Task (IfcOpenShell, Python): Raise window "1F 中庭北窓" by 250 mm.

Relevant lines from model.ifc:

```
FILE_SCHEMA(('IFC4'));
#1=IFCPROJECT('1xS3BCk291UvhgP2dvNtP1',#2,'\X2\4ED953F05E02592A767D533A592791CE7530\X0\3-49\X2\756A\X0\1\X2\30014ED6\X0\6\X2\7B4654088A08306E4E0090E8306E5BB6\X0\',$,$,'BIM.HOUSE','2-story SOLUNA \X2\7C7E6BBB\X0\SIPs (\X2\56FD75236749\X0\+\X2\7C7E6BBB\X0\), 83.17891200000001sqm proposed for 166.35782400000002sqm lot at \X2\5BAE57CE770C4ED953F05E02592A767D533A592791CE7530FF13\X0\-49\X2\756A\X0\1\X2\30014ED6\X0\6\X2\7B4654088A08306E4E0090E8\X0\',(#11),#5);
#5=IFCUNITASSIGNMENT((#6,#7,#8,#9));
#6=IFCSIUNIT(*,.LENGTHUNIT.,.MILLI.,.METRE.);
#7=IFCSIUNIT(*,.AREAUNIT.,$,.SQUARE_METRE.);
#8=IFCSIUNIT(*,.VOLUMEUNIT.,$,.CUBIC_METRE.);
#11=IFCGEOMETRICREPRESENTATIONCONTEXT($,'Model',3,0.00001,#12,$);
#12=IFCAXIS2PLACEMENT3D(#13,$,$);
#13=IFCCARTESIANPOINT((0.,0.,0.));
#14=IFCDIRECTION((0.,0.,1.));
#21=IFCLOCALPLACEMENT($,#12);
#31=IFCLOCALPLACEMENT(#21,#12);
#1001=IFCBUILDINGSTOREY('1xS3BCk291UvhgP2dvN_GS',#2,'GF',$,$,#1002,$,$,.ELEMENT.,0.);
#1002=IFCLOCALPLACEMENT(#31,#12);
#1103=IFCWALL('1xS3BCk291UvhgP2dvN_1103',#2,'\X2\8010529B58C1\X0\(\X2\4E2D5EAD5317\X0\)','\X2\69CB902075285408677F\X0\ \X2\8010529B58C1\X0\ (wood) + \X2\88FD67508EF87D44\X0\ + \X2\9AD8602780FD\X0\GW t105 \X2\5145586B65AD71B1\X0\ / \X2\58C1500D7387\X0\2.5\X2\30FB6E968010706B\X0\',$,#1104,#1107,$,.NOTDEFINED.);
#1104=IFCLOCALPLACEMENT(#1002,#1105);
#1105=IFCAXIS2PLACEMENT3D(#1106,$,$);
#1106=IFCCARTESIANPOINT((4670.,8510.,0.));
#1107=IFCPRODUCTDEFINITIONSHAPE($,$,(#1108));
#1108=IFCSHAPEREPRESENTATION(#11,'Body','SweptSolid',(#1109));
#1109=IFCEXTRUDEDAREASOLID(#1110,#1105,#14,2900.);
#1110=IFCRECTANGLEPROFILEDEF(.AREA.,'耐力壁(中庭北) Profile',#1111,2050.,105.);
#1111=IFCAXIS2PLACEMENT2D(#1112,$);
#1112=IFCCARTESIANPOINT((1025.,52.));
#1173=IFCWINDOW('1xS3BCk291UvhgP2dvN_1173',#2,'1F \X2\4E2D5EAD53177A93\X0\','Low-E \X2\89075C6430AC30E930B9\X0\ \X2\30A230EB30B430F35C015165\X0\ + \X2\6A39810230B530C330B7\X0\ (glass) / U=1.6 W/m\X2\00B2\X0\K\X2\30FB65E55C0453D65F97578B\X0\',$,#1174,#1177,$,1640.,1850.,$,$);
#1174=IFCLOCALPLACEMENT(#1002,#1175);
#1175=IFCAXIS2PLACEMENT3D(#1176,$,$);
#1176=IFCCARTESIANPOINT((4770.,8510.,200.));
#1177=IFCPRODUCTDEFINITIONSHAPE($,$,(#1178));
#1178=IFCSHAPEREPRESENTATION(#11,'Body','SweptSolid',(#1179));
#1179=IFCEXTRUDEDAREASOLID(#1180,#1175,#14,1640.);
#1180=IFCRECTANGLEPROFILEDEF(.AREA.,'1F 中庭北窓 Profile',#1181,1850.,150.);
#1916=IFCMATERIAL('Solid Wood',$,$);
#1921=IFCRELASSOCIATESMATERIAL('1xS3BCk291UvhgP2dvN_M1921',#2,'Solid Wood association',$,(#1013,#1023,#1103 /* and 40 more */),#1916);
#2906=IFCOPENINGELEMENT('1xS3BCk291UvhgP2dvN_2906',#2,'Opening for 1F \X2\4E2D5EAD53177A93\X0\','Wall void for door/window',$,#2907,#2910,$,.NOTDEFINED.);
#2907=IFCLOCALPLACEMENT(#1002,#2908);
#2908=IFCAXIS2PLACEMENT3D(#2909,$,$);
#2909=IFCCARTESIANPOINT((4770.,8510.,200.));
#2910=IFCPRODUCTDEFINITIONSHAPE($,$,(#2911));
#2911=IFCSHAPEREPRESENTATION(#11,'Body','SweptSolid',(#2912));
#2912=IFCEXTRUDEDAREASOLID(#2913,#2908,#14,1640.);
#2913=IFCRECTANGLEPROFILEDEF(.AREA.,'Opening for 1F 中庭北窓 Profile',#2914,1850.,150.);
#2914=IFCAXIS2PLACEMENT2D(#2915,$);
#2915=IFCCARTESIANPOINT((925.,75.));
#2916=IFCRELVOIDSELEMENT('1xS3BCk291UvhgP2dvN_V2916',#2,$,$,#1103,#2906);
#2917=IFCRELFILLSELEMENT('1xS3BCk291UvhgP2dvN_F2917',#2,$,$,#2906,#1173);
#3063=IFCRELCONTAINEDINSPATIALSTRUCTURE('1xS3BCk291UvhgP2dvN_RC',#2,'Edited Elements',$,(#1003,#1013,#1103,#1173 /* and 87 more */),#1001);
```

```python
import numpy as np
import ifcopenshell
import ifcopenshell.api.geometry
import ifcopenshell.util.placement
import ifcopenshell.util.unit

model = ifcopenshell.open("model.ifc")
unit_scale = ifcopenshell.util.unit.calculate_unit_scale(model)

window = model.by_guid("1xS3BCk291UvhgP2dvN_1173")
opening = window.FillsVoids[0].RelatingOpeningElement
dz = 0.25 / unit_scale

shift = np.array([0.0, 0.0, dz])
# The window is not placed relative to its opening, so move both.
for product in (opening, window):
    matrix = ifcopenshell.util.placement.get_local_placement(product.ObjectPlacement)
    matrix[:3, 3] += shift
    ifcopenshell.api.geometry.edit_object_placement(model, product=product, matrix=matrix, is_si=False)

print(f"moved by {dz * unit_scale:+.3f} m")

model.write("model_edited.ifc")
```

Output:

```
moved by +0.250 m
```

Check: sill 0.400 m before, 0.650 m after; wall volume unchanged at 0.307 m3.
